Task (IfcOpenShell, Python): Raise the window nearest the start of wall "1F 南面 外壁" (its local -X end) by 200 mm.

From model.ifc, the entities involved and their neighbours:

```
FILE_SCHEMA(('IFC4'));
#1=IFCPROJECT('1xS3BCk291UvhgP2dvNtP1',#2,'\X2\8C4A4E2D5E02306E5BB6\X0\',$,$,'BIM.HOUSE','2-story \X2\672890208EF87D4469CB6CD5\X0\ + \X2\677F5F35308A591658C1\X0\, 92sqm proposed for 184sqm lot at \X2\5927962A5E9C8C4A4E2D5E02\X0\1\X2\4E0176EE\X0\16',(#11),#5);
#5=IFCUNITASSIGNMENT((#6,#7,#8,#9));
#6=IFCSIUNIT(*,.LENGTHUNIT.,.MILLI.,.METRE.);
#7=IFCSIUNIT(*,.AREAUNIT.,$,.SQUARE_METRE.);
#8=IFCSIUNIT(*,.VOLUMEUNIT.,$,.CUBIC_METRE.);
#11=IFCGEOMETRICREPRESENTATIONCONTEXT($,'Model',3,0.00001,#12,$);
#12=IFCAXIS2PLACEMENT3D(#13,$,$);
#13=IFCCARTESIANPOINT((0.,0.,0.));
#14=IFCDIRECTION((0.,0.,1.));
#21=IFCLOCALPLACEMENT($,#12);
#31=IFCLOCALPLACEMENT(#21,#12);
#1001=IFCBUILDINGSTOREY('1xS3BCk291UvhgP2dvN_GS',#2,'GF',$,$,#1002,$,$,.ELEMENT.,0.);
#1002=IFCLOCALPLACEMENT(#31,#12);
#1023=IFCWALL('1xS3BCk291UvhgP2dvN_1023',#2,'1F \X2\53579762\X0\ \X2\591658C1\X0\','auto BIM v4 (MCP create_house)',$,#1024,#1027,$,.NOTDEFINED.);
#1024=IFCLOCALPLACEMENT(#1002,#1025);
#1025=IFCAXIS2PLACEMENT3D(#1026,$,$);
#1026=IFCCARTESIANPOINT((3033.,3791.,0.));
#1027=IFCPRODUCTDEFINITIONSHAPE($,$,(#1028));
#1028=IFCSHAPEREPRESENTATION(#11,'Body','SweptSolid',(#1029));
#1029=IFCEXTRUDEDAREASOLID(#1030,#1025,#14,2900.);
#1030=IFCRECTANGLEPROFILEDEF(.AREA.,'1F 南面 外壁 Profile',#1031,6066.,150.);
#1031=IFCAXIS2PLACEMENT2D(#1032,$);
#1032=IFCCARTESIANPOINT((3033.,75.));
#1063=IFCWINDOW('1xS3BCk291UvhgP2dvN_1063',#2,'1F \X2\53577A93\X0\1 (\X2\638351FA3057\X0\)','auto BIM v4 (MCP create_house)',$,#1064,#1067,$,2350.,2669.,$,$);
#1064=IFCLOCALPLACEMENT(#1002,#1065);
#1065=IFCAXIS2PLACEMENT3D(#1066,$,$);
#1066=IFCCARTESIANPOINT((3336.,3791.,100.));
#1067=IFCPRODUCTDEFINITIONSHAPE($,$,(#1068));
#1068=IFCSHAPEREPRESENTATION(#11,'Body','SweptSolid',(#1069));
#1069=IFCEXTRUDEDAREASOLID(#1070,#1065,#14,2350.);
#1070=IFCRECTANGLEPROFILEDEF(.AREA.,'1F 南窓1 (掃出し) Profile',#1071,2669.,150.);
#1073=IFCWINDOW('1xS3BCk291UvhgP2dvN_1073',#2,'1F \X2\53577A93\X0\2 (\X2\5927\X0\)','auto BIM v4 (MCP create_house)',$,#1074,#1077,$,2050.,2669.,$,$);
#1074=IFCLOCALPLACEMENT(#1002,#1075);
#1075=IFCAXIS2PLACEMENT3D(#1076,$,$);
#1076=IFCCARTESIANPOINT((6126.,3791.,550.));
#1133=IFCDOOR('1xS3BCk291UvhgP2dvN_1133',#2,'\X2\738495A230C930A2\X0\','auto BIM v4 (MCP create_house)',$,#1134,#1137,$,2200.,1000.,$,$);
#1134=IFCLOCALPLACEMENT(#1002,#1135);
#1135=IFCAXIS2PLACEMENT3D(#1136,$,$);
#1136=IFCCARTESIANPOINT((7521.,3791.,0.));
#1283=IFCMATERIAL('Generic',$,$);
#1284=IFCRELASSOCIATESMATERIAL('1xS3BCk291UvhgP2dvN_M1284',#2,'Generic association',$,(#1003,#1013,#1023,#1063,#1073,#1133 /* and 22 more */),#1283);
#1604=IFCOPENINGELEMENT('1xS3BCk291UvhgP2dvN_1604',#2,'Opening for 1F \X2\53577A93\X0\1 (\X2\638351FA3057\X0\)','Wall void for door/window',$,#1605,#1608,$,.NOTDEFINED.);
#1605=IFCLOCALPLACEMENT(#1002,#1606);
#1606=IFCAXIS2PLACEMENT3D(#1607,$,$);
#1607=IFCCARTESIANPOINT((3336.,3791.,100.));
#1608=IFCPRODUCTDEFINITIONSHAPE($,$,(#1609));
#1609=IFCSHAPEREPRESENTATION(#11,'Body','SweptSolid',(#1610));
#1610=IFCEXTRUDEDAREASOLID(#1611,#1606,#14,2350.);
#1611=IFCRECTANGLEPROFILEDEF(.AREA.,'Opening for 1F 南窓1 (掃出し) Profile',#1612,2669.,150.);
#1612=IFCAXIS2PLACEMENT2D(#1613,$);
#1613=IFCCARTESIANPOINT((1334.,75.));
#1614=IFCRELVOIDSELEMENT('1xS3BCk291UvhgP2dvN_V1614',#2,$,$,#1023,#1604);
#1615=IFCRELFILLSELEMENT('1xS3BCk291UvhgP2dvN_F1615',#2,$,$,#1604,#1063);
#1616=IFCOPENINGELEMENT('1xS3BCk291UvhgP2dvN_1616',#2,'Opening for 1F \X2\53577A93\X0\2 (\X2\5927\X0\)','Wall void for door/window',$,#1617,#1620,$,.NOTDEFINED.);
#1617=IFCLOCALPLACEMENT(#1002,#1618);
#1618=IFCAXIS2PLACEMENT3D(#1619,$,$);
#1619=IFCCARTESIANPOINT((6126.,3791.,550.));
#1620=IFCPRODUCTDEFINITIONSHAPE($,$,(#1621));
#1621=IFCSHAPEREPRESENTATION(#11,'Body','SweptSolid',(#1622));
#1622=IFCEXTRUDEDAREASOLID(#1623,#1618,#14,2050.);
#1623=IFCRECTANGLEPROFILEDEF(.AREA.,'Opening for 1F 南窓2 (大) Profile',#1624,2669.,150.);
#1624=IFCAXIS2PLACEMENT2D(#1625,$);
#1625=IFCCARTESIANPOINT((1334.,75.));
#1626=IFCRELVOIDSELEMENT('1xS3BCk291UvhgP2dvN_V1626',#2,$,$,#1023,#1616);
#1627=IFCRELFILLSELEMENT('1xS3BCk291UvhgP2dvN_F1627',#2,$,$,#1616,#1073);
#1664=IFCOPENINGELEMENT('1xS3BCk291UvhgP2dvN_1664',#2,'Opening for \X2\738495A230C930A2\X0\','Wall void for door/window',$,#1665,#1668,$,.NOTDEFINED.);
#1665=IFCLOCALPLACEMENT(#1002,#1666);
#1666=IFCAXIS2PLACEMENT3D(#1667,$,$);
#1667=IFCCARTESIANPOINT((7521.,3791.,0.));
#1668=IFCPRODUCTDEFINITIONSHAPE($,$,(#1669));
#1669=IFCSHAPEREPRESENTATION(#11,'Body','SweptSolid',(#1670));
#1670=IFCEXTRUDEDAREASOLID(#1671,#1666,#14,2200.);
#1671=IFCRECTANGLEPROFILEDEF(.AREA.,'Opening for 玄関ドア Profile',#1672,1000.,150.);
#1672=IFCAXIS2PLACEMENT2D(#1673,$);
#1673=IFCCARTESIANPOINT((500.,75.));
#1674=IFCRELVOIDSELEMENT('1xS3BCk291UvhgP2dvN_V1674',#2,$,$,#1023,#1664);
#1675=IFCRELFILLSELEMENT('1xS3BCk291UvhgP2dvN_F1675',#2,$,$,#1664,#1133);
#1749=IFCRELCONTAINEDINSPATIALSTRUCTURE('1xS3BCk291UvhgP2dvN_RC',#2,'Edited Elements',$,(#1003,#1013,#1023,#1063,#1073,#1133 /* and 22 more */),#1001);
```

```python
import numpy as np
import ifcopenshell
import ifcopenshell.api.geometry
import ifcopenshell.util.placement
import ifcopenshell.util.unit

model = ifcopenshell.open("model.ifc")
unit_scale = ifcopenshell.util.unit.calculate_unit_scale(model)

window = model.by_guid("1xS3BCk291UvhgP2dvN_1063")
opening = window.FillsVoids[0].RelatingOpeningElement
dz = 0.2 / unit_scale

shift = np.array([0.0, 0.0, dz])
# The window is not placed relative to its opening, so move both.
for product in (opening, window):
    matrix = ifcopenshell.util.placement.get_local_placement(product.ObjectPlacement)
    matrix[:3, 3] += shift
    ifcopenshell.api.geometry.edit_object_placement(model, product=product, matrix=matrix, is_si=False)

print(f"moved by {dz * unit_scale:+.3f} m")

model.write("model_rev.ifc")
```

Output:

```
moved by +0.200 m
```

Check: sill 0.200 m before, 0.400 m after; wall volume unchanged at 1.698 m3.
